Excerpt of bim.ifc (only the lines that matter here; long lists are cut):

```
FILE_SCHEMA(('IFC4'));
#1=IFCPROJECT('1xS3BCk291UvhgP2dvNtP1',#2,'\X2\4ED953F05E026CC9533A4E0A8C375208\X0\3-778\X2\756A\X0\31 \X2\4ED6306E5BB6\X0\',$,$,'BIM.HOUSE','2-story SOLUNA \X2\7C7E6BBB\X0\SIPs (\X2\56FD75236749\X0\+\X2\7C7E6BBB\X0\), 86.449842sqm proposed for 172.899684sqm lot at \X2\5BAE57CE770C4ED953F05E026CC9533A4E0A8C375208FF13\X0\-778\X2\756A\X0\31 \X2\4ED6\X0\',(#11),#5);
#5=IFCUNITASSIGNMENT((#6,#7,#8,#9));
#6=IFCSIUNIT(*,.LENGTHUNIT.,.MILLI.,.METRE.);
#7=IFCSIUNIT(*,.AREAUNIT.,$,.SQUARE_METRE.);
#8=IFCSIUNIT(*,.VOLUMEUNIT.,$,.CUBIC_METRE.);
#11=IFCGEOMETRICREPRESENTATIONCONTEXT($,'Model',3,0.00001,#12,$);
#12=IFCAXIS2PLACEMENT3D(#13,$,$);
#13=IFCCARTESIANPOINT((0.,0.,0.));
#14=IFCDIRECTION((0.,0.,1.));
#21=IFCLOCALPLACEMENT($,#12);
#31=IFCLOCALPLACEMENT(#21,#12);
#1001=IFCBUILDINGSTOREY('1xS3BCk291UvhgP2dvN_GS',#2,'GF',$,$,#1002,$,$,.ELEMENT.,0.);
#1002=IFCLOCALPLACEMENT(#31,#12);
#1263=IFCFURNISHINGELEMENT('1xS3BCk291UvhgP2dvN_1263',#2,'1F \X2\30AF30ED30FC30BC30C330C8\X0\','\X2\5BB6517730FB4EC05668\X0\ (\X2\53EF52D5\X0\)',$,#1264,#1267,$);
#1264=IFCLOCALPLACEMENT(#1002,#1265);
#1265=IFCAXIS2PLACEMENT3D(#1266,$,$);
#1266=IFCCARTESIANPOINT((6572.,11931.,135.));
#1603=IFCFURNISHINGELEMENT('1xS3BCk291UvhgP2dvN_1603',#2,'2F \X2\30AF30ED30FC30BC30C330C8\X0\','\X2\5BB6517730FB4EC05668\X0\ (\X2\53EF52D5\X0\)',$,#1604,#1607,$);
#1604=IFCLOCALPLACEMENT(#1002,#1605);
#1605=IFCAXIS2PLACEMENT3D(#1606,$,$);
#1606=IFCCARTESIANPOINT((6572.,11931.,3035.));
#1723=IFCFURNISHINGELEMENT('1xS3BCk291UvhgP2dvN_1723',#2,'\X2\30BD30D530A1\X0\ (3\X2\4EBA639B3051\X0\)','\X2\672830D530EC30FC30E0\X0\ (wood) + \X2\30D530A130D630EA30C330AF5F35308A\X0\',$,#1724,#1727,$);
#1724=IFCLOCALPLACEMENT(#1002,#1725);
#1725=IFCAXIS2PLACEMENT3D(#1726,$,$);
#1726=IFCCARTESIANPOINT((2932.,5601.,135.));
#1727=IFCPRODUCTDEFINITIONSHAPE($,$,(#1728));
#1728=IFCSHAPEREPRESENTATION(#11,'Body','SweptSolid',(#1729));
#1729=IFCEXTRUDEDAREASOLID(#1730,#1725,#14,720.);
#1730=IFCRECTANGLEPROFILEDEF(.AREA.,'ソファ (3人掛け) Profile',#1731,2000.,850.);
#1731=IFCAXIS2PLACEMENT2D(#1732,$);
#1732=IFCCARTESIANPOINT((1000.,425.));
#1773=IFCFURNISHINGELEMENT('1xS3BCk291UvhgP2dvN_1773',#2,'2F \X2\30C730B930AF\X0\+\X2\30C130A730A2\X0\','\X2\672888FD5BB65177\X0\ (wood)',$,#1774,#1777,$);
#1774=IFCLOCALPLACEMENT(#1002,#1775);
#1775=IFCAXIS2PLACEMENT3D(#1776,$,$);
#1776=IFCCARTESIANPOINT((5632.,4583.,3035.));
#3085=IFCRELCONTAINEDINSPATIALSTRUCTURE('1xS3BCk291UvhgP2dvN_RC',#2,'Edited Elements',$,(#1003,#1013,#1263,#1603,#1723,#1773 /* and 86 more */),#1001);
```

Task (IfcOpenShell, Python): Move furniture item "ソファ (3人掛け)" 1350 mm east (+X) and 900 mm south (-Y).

```python
import ifcopenshell
import ifcopenshell.api.geometry
import ifcopenshell.util.placement
import ifcopenshell.util.unit

model = ifcopenshell.open("bim.ifc")
unit_scale = ifcopenshell.util.unit.calculate_unit_scale(model)

item = model.by_guid("1xS3BCk291UvhgP2dvN_1723")
matrix = ifcopenshell.util.placement.get_local_placement(item.ObjectPlacement)
matrix[0, 3] += 1.35 / unit_scale
matrix[1, 3] -= 0.9 / unit_scale
ifcopenshell.api.geometry.edit_object_placement(model, product=item, matrix=matrix, is_si=False)

print(ifcopenshell.util.placement.get_local_placement(item.ObjectPlacement).round(3) + 0.0)

model.write("bim-out.ifc")
```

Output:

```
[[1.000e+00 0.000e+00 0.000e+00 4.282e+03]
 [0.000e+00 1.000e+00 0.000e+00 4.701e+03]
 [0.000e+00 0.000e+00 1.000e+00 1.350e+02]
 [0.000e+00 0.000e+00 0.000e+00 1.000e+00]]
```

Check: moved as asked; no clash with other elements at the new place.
